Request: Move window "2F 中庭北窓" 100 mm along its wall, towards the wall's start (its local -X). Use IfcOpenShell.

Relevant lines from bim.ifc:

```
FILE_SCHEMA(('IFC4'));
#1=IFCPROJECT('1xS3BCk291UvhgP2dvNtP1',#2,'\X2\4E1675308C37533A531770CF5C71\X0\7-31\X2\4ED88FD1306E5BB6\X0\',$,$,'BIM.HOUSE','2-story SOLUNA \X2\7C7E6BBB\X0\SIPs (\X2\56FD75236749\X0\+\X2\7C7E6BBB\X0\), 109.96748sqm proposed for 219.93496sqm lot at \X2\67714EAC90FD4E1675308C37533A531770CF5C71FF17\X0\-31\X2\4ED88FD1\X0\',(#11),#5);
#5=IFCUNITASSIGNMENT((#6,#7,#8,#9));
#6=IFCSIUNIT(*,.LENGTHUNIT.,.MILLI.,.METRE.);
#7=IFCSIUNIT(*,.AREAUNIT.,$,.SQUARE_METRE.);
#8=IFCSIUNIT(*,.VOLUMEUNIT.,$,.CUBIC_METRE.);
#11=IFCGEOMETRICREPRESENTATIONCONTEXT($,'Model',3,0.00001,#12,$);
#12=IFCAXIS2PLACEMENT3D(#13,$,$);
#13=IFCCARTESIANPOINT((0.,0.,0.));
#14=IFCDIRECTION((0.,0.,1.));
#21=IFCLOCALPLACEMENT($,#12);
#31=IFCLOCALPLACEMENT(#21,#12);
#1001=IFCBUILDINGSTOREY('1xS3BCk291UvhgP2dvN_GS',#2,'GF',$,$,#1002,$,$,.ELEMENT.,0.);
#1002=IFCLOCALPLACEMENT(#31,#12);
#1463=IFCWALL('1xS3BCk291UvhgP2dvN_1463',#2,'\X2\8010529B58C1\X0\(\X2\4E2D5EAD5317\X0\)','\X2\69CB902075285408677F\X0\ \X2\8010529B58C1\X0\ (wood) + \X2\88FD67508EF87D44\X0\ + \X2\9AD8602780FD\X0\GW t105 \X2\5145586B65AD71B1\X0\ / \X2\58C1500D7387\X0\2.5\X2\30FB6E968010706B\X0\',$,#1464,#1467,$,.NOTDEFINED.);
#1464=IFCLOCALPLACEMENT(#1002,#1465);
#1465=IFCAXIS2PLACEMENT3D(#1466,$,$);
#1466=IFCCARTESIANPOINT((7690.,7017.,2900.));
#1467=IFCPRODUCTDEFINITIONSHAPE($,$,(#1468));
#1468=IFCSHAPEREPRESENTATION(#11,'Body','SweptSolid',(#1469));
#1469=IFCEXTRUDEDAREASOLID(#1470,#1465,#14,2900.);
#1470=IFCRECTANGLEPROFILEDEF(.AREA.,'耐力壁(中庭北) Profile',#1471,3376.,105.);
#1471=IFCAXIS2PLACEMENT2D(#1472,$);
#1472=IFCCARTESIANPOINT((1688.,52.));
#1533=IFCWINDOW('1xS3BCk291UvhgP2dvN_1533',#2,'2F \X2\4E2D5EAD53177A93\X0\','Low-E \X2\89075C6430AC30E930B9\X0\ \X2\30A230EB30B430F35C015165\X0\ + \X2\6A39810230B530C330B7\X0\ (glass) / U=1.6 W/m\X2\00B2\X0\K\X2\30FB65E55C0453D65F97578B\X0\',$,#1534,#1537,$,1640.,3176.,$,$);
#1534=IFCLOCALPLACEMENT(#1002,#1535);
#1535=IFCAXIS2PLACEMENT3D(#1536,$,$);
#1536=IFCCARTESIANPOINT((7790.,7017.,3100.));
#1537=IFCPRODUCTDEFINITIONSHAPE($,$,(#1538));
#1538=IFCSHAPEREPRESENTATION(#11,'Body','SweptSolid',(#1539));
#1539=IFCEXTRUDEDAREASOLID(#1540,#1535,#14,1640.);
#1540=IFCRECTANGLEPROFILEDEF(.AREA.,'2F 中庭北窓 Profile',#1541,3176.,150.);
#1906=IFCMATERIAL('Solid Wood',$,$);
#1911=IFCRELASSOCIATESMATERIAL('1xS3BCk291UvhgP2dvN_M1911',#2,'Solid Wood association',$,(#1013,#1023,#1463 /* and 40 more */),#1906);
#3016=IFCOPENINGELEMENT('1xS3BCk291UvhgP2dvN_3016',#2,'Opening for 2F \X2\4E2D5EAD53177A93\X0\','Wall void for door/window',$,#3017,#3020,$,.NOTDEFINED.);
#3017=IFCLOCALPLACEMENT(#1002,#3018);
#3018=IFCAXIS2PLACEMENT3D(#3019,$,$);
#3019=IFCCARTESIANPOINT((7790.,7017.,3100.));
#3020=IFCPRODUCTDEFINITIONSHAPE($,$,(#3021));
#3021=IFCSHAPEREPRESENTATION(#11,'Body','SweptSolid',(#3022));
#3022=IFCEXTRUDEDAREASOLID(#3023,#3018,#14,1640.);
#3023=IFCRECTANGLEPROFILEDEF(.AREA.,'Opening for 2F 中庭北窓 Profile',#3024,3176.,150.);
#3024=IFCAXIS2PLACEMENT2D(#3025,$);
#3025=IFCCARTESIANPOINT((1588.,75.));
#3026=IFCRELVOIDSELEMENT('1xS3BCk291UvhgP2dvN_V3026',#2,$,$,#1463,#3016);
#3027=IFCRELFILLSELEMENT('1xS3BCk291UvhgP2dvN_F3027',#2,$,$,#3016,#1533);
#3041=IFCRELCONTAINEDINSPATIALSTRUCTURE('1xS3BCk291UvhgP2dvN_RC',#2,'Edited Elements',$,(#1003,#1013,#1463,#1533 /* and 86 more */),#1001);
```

```python
import ifcopenshell
import ifcopenshell.api.geometry
import ifcopenshell.util.placement

model = ifcopenshell.open("bim.ifc")

window = model.by_guid("1xS3BCk291UvhgP2dvN_1533")
opening = window.FillsVoids[0].RelatingOpeningElement
wall = opening.VoidsElements[0].RelatingBuildingElement

wall_matrix = ifcopenshell.util.placement.get_local_placement(wall.ObjectPlacement)
shift = wall_matrix[:3, 0] * -100.0
before = ifcopenshell.util.placement.get_local_placement(window.ObjectPlacement)[:3, 3].copy()

# The window is not placed relative to its opening, so move both.
for product in (opening, window):
    matrix = ifcopenshell.util.placement.get_local_placement(product.ObjectPlacement)
    matrix[:3, 3] += shift
    ifcopenshell.api.geometry.edit_object_placement(model, product=product, matrix=matrix, is_si=False)

after = ifcopenshell.util.placement.get_local_placement(window.ObjectPlacement)[:3, 3]
print("window moved by", (after - before).round(3) + 0.0)

model.write("bim_updated.ifc")
```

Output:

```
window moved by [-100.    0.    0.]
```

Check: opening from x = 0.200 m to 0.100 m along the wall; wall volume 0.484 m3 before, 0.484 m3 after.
